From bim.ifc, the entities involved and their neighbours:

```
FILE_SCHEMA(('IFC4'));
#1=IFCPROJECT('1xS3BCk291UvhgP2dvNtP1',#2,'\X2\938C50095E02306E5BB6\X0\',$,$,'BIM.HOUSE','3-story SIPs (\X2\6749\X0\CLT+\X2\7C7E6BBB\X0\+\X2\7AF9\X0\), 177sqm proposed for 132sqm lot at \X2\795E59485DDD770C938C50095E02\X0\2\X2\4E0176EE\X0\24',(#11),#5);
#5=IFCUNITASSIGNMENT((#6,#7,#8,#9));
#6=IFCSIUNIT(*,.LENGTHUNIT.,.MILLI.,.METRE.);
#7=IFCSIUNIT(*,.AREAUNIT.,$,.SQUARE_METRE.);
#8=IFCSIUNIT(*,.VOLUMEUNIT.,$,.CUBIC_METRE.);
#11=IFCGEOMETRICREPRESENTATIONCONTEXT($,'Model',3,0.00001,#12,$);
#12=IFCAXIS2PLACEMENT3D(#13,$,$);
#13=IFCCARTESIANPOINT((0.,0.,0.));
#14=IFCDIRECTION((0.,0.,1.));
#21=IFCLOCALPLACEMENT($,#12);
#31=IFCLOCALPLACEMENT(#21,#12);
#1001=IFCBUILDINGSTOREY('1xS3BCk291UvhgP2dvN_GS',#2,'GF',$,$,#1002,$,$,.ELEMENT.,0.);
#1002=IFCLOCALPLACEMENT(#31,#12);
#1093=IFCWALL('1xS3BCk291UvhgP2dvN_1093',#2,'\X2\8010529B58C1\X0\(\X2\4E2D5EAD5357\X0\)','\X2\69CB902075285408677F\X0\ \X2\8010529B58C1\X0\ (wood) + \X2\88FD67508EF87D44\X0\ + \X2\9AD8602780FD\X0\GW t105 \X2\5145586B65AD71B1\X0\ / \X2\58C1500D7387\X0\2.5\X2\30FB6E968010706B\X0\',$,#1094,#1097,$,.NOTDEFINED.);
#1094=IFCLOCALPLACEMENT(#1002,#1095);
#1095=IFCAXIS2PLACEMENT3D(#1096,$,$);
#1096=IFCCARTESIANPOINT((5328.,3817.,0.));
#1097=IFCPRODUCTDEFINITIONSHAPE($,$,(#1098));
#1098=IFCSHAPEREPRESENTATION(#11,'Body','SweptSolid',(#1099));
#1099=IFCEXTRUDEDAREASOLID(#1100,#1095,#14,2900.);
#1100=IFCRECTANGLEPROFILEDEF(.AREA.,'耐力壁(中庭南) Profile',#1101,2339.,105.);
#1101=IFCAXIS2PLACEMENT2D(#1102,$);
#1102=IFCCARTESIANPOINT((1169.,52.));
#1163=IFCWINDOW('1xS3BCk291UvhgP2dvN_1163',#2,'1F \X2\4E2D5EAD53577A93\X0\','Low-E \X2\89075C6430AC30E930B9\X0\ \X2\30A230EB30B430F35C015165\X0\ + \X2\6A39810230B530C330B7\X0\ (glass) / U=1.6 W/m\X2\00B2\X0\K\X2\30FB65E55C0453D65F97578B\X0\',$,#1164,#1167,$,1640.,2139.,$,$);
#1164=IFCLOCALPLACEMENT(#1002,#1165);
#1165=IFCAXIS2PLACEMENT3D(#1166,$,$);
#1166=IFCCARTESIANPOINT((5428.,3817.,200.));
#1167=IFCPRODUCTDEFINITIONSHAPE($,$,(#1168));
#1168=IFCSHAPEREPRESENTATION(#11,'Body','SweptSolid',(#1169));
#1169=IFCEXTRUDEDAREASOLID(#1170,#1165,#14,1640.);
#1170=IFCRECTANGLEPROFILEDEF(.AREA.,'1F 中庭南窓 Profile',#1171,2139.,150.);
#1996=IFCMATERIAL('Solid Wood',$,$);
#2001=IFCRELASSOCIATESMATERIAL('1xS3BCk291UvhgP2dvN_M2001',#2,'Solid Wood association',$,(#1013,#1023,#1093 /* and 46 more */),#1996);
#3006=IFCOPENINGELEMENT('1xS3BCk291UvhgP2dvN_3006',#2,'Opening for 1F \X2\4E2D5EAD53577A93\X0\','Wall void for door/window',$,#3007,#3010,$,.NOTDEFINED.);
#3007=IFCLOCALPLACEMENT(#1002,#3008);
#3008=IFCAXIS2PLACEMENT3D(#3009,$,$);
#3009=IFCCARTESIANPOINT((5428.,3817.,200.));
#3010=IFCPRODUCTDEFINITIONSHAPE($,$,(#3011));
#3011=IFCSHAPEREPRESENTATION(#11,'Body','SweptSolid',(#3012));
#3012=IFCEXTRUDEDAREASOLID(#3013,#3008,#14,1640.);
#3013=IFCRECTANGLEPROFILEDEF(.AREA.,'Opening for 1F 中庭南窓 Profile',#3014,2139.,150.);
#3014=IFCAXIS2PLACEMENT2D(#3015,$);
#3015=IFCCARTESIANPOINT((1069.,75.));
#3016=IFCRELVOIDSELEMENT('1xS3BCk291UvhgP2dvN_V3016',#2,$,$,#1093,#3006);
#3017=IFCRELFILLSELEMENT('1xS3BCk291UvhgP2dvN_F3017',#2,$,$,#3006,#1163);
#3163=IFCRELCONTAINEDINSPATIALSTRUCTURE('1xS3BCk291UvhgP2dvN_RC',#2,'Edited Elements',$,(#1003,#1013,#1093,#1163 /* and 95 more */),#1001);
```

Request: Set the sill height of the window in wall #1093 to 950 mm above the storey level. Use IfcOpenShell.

```python
import numpy as np
import ifcopenshell
import ifcopenshell.api.geometry
import ifcopenshell.geom
import ifcopenshell.util.element
import ifcopenshell.util.placement
import ifcopenshell.util.shape
import ifcopenshell.util.unit

model = ifcopenshell.open("bim.ifc")
unit_scale = ifcopenshell.util.unit.calculate_unit_scale(model)

window = model.by_guid("1xS3BCk291UvhgP2dvN_1163")
opening = window.FillsVoids[0].RelatingOpeningElement
storey = ifcopenshell.util.element.get_container(window, ifc_class="IfcBuildingStorey")
level = ifcopenshell.util.placement.get_local_placement(storey.ObjectPlacement)[2, 3]

# The opening's origin need not be at the sill, so measure its lowest point.
shape = ifcopenshell.geom.create_shape(ifcopenshell.geom.settings(), opening)
bottom = ifcopenshell.util.shape.get_shape_bottom_elevation(shape, shape.geometry) / unit_scale
dz = level + 0.95 / unit_scale - bottom

shift = np.array([0.0, 0.0, dz])
# The window is not placed relative to its opening, so move both.
for product in (opening, window):
    matrix = ifcopenshell.util.placement.get_local_placement(product.ObjectPlacement)
    matrix[:3, 3] += shift
    ifcopenshell.api.geometry.edit_object_placement(model, product=product, matrix=matrix, is_si=False)

print(f"moved by {dz * unit_scale:+.3f} m")

model.write("bim-out.ifc")
```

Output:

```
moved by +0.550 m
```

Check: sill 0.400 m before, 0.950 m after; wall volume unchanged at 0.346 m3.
